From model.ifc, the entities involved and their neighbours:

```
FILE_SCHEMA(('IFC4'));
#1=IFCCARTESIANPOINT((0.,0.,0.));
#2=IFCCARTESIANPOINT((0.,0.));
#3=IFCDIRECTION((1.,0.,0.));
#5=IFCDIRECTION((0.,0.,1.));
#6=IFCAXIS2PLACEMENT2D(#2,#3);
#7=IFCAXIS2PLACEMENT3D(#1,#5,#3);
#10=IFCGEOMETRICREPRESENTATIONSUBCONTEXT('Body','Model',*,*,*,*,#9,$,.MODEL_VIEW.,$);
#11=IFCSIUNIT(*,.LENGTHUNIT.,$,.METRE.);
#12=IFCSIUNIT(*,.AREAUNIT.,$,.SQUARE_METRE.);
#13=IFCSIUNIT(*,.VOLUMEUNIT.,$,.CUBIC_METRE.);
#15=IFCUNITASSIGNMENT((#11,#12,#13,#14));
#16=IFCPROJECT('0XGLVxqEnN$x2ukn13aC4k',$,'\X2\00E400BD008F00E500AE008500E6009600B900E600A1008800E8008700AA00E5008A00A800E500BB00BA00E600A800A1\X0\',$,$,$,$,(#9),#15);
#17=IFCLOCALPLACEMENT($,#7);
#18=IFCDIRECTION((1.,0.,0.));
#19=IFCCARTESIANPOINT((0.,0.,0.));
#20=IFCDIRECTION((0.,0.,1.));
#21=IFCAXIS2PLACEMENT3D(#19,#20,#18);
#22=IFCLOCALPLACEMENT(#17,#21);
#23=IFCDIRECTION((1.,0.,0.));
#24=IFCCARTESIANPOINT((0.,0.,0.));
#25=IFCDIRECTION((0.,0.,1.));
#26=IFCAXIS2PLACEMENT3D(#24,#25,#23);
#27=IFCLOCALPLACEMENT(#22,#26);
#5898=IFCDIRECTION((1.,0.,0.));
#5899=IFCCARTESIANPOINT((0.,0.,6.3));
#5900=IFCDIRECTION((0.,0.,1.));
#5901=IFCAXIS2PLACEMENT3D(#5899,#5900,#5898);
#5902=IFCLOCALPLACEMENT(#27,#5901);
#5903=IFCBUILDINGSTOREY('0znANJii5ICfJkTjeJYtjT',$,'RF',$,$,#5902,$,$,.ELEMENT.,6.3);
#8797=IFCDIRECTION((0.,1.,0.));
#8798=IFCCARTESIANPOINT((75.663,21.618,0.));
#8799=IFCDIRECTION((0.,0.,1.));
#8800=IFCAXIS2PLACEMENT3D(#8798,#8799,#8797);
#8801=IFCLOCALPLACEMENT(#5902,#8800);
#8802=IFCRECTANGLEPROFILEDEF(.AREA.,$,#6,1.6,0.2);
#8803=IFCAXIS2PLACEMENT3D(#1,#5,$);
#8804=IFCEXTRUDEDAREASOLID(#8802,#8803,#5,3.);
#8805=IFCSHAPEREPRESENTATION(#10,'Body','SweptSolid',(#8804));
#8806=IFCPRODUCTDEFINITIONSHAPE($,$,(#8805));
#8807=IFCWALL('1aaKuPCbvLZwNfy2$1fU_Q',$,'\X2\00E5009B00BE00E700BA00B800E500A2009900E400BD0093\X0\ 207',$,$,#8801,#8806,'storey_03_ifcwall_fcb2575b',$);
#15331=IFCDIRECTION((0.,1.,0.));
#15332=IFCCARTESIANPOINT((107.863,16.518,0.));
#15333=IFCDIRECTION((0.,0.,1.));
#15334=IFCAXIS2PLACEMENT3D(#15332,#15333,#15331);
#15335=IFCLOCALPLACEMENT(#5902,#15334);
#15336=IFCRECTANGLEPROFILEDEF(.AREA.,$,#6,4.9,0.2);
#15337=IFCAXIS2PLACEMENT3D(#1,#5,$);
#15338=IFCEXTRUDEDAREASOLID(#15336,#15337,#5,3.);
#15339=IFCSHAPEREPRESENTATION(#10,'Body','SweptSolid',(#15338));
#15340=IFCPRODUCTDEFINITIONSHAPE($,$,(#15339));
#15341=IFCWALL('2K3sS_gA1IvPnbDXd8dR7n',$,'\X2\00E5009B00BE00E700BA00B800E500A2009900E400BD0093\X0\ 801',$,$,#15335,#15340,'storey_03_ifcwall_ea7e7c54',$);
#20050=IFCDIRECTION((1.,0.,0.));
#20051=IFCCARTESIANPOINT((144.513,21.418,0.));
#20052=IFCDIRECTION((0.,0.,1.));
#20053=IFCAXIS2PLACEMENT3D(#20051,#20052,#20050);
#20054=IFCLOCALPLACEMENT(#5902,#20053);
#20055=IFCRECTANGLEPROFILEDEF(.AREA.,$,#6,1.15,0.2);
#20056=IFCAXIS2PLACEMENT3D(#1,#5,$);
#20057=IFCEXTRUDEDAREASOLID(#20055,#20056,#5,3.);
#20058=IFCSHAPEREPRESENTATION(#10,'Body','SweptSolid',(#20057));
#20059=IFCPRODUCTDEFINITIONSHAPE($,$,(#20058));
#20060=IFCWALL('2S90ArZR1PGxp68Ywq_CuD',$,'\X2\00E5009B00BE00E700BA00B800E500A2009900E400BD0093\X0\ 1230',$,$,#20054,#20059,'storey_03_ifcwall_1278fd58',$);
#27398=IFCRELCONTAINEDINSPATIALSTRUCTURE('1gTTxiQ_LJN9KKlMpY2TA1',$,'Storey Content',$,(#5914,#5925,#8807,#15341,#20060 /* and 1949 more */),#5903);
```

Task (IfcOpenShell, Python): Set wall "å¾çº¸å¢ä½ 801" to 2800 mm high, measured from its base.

```python
import ifcopenshell
import ifcopenshell.geom
import ifcopenshell.util.representation
import ifcopenshell.util.shape
import ifcopenshell.util.unit

model = ifcopenshell.open("model.ifc")
unit_scale = ifcopenshell.util.unit.calculate_unit_scale(model)
settings = ifcopenshell.geom.settings()


def volume(element):
    """Net volume in cubic metres, openings subtracted."""
    shape = ifcopenshell.geom.create_shape(settings, element)
    return ifcopenshell.util.shape.get_volume(shape.geometry)


wall = model.by_guid("2K3sS_gA1IvPnbDXd8dR7n")
before = volume(wall)

body = ifcopenshell.util.representation.get_representation(wall, "Model", "Body")
solid = body.Items[0]
old_height = solid.Depth
solid.Depth = 2.8 / unit_scale
after = volume(wall)

print(f"height {old_height:g} -> {solid.Depth:g}, volume {before:.3f} -> {after:.3f} m3")

model.write("model_rev.ifc")
```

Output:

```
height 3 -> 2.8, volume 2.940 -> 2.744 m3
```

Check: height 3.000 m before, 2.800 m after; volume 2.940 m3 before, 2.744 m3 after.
